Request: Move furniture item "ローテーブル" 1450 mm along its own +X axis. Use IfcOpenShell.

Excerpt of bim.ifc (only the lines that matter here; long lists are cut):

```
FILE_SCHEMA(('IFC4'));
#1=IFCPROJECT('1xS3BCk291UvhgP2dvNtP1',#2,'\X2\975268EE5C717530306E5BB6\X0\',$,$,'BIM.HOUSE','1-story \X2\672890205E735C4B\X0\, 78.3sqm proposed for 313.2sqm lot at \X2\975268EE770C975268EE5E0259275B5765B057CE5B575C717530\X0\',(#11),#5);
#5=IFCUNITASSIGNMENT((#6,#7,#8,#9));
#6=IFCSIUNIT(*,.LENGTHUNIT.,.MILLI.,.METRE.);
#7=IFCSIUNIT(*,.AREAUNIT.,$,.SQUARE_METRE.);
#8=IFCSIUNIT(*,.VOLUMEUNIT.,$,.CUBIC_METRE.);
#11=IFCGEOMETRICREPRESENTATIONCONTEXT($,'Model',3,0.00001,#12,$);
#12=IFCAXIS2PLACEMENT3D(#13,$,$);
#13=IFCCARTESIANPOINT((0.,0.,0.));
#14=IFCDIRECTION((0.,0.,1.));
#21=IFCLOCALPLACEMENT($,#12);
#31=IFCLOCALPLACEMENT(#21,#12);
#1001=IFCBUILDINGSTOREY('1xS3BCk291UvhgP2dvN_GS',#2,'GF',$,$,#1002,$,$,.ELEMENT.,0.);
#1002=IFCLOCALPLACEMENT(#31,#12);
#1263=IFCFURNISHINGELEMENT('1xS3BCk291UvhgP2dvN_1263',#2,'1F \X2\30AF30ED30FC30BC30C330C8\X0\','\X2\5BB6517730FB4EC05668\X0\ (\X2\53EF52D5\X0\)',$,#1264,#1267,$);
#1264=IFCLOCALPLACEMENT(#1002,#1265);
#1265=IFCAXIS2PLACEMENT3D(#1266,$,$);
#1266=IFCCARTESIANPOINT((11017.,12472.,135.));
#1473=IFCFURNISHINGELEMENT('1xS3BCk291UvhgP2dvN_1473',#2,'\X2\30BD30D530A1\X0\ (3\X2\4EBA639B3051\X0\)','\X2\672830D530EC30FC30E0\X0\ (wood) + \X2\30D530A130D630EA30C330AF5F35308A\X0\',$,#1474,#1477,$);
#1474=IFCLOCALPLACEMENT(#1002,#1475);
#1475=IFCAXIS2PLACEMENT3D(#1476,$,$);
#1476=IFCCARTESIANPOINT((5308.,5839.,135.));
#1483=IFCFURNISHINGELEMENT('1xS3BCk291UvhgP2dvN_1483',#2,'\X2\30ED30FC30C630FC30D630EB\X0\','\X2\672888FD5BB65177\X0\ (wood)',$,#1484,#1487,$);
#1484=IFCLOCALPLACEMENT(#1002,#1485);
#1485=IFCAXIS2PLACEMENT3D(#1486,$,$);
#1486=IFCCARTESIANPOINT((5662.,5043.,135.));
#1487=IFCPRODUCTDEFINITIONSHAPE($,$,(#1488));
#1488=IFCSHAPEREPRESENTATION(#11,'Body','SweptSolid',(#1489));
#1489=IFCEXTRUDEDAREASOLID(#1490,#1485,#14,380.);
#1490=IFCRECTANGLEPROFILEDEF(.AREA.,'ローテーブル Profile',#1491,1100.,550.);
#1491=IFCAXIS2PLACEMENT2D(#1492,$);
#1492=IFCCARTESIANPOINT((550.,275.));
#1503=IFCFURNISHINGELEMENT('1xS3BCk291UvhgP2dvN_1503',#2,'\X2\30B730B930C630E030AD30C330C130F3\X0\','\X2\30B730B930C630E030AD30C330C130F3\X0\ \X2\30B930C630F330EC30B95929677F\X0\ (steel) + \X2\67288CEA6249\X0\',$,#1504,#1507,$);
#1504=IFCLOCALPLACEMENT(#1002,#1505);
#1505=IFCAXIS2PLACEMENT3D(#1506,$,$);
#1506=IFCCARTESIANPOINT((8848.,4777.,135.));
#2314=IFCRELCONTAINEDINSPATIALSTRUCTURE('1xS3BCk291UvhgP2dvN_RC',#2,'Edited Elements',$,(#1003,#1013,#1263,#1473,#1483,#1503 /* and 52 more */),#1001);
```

```python
import ifcopenshell
import ifcopenshell.api.geometry
import ifcopenshell.util.placement
import ifcopenshell.util.unit

model = ifcopenshell.open("bim.ifc")
unit_scale = ifcopenshell.util.unit.calculate_unit_scale(model)

item = model.by_guid("1xS3BCk291UvhgP2dvN_1483")
matrix = ifcopenshell.util.placement.get_local_placement(item.ObjectPlacement)
matrix[:3, 3] += matrix[:3, 0] * 1.45 / unit_scale
ifcopenshell.api.geometry.edit_object_placement(model, product=item, matrix=matrix, is_si=False)

print(ifcopenshell.util.placement.get_local_placement(item.ObjectPlacement).round(3) + 0.0)

model.write("bim_v2.ifc")
```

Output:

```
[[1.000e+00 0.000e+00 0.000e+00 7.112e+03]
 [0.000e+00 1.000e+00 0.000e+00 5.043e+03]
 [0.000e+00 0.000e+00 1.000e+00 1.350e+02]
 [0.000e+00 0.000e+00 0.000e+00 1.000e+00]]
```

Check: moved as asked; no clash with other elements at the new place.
